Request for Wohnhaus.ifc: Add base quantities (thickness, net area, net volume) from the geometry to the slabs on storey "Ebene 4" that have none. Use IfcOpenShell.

First a look at what the model holds.

```python
import ifcopenshell
import ifcopenshell.util.element
import ifcopenshell.util.unit

model = ifcopenshell.open("Wohnhaus.ifc")
print(model.schema)
for unit_type in ("LENGTHUNIT", "AREAUNIT", "VOLUMEUNIT"):
    print(unit_type, ifcopenshell.util.unit.calculate_unit_scale(model, unit_type))
storey = next(s for s in model.by_type("IfcBuildingStorey") if s.Name == "Ebene 4")
slabs = [e for e in ifcopenshell.util.element.get_decomposition(storey) if e.is_a("IfcSlab")]
for e in sorted(slabs, key=lambda e: e.id()):
    print(e.id(), e.is_a(), e.Name, list(ifcopenshell.util.element.get_psets(e, qtos_only=True)), sep=" | ")
```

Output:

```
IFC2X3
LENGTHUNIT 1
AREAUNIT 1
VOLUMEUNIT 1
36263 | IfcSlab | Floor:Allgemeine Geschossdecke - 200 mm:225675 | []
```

```python
import ifcopenshell
import ifcopenshell.api.pset
import ifcopenshell.geom
import ifcopenshell.util.element
import ifcopenshell.util.shape
import ifcopenshell.util.unit

model = ifcopenshell.open("Wohnhaus.ifc")
unit_scale = ifcopenshell.util.unit.calculate_unit_scale(model)
area_scale = ifcopenshell.util.unit.calculate_unit_scale(model, "AREAUNIT")
volume_scale = ifcopenshell.util.unit.calculate_unit_scale(model, "VOLUMEUNIT")
settings = ifcopenshell.geom.settings()

storey = next(s for s in model.by_type("IfcBuildingStorey") if s.Name == "Ebene 4")
slabs = [e for e in ifcopenshell.util.element.get_decomposition(storey) if e.is_a("IfcSlab")]

for e in sorted(slabs, key=lambda e: e.id()):
    if ifcopenshell.util.element.get_psets(e, qtos_only=True, should_inherit=False):
        continue
    # Geometry comes back in metres, in the element's own axes.
    shape = ifcopenshell.geom.create_shape(settings, e)
    values = {
        "Width": ifcopenshell.util.shape.get_z(shape.geometry) / unit_scale,
        "NetArea": ifcopenshell.util.shape.get_footprint_area(shape.geometry) / area_scale,
        "NetVolume": ifcopenshell.util.shape.get_volume(shape.geometry) / volume_scale,
    }
    qto = ifcopenshell.api.pset.add_qto(model, product=e, name="BaseQuantities")
    ifcopenshell.api.pset.edit_qto(model, qto=qto, properties=values)
    print(e.id(), {k: round(v, 3) for k, v in values.items()})

model.write("Wohnhaus_updated.ifc")
```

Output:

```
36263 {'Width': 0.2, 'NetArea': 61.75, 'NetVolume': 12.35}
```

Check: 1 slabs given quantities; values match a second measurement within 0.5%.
